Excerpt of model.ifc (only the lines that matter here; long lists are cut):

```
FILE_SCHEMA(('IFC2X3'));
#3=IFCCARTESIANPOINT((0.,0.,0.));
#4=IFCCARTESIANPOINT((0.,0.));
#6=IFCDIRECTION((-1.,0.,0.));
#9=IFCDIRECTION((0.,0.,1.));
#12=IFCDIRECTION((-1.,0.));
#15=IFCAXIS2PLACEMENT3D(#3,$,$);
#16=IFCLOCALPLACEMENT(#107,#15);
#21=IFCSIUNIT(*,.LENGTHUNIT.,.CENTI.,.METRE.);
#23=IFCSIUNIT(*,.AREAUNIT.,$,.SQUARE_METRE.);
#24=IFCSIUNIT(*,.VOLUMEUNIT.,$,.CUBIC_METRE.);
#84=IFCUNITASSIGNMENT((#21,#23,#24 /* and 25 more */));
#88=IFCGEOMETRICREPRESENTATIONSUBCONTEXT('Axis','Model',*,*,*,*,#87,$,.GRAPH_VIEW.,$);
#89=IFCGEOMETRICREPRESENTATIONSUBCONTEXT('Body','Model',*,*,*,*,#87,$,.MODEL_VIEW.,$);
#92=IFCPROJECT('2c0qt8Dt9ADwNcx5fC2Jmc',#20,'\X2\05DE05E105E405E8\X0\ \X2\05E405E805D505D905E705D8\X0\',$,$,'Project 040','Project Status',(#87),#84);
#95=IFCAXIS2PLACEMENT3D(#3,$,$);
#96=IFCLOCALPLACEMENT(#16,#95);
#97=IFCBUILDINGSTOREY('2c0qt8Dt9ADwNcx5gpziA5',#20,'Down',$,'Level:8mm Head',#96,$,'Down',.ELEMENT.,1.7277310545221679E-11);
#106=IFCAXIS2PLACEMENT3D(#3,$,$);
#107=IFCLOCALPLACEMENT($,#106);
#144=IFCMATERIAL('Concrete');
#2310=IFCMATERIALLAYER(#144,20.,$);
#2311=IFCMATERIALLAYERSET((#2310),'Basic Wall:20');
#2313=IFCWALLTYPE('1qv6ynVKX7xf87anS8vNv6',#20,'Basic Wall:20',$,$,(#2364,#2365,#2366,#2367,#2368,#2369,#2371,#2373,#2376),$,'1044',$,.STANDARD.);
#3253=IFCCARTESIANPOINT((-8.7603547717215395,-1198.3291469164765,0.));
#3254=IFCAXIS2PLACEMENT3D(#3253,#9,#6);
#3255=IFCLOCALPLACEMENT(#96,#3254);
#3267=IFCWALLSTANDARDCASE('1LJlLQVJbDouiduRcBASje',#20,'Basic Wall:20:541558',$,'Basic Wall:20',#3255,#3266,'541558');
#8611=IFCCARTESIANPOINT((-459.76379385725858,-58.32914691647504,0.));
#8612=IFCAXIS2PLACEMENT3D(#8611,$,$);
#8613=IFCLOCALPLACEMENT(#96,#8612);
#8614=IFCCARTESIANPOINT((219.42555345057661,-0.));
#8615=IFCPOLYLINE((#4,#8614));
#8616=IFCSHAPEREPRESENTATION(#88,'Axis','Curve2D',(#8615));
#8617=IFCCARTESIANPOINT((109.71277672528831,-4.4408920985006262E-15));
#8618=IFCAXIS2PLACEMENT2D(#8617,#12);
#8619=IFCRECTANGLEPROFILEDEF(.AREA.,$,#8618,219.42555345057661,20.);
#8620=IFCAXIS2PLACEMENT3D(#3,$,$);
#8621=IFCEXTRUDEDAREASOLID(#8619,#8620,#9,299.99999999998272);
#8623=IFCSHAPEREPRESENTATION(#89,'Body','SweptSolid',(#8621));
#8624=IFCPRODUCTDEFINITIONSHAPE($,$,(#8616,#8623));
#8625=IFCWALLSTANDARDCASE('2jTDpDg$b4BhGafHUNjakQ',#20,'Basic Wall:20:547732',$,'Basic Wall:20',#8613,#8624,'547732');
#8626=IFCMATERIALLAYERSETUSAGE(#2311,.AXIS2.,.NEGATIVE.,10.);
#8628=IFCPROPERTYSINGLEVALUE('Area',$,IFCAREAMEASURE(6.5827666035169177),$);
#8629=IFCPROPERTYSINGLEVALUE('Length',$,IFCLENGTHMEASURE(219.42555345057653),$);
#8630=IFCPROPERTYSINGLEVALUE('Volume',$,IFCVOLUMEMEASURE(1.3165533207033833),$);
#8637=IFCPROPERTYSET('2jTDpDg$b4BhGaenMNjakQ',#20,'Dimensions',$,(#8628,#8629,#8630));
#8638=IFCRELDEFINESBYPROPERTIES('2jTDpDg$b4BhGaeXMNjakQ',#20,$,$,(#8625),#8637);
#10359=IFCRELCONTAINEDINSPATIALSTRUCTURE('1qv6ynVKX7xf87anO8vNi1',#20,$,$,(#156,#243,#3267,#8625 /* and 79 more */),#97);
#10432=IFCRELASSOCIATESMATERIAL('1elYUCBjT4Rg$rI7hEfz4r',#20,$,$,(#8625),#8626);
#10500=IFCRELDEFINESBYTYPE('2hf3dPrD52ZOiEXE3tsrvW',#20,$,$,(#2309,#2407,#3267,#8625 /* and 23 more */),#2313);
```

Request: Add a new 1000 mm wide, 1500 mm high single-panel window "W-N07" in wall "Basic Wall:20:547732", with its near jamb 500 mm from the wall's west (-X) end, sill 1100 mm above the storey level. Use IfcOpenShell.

```python
import numpy as np
import ifcopenshell
import ifcopenshell.api.feature
import ifcopenshell.api.geometry
import ifcopenshell.api.pset
import ifcopenshell.api.root
import ifcopenshell.api.spatial
import ifcopenshell.api.type
import ifcopenshell.geom
import ifcopenshell.util.element
import ifcopenshell.util.placement
import ifcopenshell.util.representation
import ifcopenshell.util.shape
import ifcopenshell.util.unit

model = ifcopenshell.open("model.ifc")
unit_scale = ifcopenshell.util.unit.calculate_unit_scale(model)
area_scale = ifcopenshell.util.unit.calculate_unit_scale(model, "AREAUNIT")
volume_scale = ifcopenshell.util.unit.calculate_unit_scale(model, "VOLUMEUNIT")
settings = ifcopenshell.geom.settings()


def volume(element):
    """Net volume in cubic metres, openings subtracted."""
    shape = ifcopenshell.geom.create_shape(settings, element)
    return ifcopenshell.util.shape.get_volume(shape.geometry)


wall = model.by_id(8625)
storey = ifcopenshell.util.element.get_container(wall, ifc_class="IfcBuildingStorey")
context = ifcopenshell.util.representation.get_context(model, "Model", "Body", "MODEL_VIEW")
before = volume(wall)

width, height, from_end, sill = 1, 1.5, 0.5, 1.1  # metres

# The wall runs along its own X axis, and the end named is its -X end.
wall_shape = ifcopenshell.geom.create_shape(settings, wall)
x, y, z = ifcopenshell.util.shape.get_vertices(wall_shape.geometry).T
start = x.min() + from_end
face, thickness = float(y.min()), float(y.max() - y.min())
wall_matrix = ifcopenshell.util.placement.get_local_placement(wall.ObjectPlacement)
level = ifcopenshell.util.placement.get_local_placement(storey.ObjectPlacement)[2, 3]


def in_wall(x, y):
    """Placement at x, y metres in the wall's axes, at sill height."""
    matrix = wall_matrix.copy()
    matrix[:, 3] = wall_matrix @ np.array([x / unit_scale, y / unit_scale, 0.0, 1.0])
    matrix[2, 3] = level + sill / unit_scale
    return matrix


# Opening: a box that overshoots both wall faces by 50 mm.
opening = ifcopenshell.api.root.create_entity(model, ifc_class="IfcOpeningElement")
box = ifcopenshell.api.geometry.add_wall_representation(
    model, context=context, length=width, height=height, thickness=thickness + 0.1
)
ifcopenshell.api.geometry.assign_representation(model, product=opening, representation=box)
ifcopenshell.api.geometry.edit_object_placement(model, product=opening, matrix=in_wall(start, face - 0.05), is_si=False)
ifcopenshell.api.feature.add_feature(model, feature=opening, element=wall)

window = ifcopenshell.api.root.create_entity(model, ifc_class="IfcWindow", name="W-N07")
window.OverallWidth, window.OverallHeight = width / unit_scale, height / unit_scale
body = ifcopenshell.api.geometry.add_window_representation(
    model,
    context=context,
    overall_width=window.OverallWidth,
    overall_height=window.OverallHeight,
    partition_type="SINGLE_PANEL",
)
ifcopenshell.api.geometry.assign_representation(model, product=window, representation=body)
ifcopenshell.api.spatial.assign_container(model, products=[window], relating_structure=storey)
fills = ifcopenshell.api.feature.add_filling(model, opening=opening, element=window)
fills.OwnerHistory = window.OwnerHistory  # required in IFC2X3

# IFC2X3 keeps the operation on the window style.
style = ifcopenshell.api.root.create_entity(model, ifc_class="IfcWindowStyle", name="W-N07")
style.OperationType, style.ConstructionType = "SINGLE_PANEL", "NOTDEFINED"
style.ParameterTakesPrecedence = style.Sizeable = False
ifcopenshell.api.type.assign_type(model, related_objects=[window], relating_type=style)

# Centre the window in the wall's thickness.
ifcopenshell.api.geometry.edit_object_placement(model, product=window, matrix=in_wall(start, face), is_si=False)
window_shape = ifcopenshell.geom.create_shape(settings, window)
depth = ifcopenshell.util.shape.get_vertices(window_shape.geometry)[:, 1]
offset = face + thickness / 2 - (depth.min() + depth.max()) / 2
ifcopenshell.api.geometry.edit_object_placement(model, product=window, matrix=in_wall(start, offset), is_si=False)

after = volume(wall)

# Update the wall's stored quantities.
pset = model.by_id(ifcopenshell.util.element.get_pset(wall, "Dimensions", should_inherit=False)["id"])
ifcopenshell.api.pset.edit_pset(model, pset=pset, properties={
    "Area": model.create_entity("IfcAreaMeasure", after / thickness / area_scale),
    "Volume": model.create_entity("IfcVolumeMeasure", after / volume_scale),
})

print(f"wall volume {before:.3f} -> {after:.3f} m3")

model.write("model_v2.ifc")
```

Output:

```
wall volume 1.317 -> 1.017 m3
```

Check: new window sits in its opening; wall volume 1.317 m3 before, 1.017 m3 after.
